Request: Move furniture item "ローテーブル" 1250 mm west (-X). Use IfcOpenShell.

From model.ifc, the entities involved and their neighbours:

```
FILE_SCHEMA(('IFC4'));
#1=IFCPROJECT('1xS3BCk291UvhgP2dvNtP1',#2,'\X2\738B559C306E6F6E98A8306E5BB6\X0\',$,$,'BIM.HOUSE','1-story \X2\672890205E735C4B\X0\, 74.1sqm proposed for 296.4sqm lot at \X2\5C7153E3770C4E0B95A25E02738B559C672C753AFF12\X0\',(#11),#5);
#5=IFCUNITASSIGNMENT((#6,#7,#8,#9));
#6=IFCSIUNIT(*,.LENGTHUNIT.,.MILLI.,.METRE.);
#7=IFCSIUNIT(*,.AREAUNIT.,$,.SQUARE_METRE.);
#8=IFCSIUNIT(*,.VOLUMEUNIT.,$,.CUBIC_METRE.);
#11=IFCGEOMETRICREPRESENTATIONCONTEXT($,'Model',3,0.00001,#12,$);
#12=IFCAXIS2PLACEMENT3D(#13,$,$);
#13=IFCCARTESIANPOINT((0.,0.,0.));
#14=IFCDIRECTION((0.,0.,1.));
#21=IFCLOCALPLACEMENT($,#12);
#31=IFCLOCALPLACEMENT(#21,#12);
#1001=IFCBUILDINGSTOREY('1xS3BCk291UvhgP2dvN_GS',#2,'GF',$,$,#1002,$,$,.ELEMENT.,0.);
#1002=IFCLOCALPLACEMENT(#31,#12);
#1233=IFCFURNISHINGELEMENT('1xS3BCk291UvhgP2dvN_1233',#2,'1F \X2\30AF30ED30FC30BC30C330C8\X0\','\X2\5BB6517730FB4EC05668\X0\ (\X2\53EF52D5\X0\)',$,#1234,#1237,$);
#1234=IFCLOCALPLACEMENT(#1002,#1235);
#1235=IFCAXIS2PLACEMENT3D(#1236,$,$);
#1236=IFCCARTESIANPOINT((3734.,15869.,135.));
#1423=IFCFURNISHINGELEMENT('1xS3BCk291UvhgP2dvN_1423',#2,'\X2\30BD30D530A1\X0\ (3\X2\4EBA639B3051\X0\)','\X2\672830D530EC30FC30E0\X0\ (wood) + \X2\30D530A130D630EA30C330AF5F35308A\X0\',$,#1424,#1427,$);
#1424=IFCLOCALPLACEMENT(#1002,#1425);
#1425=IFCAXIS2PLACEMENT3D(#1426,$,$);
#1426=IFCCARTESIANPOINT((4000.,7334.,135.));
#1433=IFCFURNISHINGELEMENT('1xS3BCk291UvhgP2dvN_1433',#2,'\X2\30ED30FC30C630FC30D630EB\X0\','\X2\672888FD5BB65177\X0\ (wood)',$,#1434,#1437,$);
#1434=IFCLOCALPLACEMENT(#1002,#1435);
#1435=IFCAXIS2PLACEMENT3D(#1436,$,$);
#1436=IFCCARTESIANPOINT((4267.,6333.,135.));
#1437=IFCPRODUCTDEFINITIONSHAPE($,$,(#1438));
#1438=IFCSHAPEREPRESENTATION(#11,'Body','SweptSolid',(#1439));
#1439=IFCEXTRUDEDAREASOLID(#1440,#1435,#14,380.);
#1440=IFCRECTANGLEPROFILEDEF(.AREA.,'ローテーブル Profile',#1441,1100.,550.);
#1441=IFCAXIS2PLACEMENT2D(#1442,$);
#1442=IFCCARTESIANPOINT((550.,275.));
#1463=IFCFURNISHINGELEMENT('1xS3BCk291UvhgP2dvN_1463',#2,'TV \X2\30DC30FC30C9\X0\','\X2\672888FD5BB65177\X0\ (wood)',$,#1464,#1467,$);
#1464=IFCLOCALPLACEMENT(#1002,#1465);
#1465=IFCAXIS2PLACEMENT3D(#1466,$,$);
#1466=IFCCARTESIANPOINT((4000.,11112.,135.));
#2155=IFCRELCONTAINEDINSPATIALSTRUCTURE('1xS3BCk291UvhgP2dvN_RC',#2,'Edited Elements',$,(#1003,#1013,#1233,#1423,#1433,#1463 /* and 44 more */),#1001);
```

```python
import ifcopenshell
import ifcopenshell.api.geometry
import ifcopenshell.util.placement
import ifcopenshell.util.unit

model = ifcopenshell.open("model.ifc")
unit_scale = ifcopenshell.util.unit.calculate_unit_scale(model)

item = model.by_guid("1xS3BCk291UvhgP2dvN_1433")
matrix = ifcopenshell.util.placement.get_local_placement(item.ObjectPlacement)
matrix[0, 3] -= 1.25 / unit_scale
ifcopenshell.api.geometry.edit_object_placement(model, product=item, matrix=matrix, is_si=False)

print(ifcopenshell.util.placement.get_local_placement(item.ObjectPlacement).round(3) + 0.0)

model.write("model_updated.ifc")
```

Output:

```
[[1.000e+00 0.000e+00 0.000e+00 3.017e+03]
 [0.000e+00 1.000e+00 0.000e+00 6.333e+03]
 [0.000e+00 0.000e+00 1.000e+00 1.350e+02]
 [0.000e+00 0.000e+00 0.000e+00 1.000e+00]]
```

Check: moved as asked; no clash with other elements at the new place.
